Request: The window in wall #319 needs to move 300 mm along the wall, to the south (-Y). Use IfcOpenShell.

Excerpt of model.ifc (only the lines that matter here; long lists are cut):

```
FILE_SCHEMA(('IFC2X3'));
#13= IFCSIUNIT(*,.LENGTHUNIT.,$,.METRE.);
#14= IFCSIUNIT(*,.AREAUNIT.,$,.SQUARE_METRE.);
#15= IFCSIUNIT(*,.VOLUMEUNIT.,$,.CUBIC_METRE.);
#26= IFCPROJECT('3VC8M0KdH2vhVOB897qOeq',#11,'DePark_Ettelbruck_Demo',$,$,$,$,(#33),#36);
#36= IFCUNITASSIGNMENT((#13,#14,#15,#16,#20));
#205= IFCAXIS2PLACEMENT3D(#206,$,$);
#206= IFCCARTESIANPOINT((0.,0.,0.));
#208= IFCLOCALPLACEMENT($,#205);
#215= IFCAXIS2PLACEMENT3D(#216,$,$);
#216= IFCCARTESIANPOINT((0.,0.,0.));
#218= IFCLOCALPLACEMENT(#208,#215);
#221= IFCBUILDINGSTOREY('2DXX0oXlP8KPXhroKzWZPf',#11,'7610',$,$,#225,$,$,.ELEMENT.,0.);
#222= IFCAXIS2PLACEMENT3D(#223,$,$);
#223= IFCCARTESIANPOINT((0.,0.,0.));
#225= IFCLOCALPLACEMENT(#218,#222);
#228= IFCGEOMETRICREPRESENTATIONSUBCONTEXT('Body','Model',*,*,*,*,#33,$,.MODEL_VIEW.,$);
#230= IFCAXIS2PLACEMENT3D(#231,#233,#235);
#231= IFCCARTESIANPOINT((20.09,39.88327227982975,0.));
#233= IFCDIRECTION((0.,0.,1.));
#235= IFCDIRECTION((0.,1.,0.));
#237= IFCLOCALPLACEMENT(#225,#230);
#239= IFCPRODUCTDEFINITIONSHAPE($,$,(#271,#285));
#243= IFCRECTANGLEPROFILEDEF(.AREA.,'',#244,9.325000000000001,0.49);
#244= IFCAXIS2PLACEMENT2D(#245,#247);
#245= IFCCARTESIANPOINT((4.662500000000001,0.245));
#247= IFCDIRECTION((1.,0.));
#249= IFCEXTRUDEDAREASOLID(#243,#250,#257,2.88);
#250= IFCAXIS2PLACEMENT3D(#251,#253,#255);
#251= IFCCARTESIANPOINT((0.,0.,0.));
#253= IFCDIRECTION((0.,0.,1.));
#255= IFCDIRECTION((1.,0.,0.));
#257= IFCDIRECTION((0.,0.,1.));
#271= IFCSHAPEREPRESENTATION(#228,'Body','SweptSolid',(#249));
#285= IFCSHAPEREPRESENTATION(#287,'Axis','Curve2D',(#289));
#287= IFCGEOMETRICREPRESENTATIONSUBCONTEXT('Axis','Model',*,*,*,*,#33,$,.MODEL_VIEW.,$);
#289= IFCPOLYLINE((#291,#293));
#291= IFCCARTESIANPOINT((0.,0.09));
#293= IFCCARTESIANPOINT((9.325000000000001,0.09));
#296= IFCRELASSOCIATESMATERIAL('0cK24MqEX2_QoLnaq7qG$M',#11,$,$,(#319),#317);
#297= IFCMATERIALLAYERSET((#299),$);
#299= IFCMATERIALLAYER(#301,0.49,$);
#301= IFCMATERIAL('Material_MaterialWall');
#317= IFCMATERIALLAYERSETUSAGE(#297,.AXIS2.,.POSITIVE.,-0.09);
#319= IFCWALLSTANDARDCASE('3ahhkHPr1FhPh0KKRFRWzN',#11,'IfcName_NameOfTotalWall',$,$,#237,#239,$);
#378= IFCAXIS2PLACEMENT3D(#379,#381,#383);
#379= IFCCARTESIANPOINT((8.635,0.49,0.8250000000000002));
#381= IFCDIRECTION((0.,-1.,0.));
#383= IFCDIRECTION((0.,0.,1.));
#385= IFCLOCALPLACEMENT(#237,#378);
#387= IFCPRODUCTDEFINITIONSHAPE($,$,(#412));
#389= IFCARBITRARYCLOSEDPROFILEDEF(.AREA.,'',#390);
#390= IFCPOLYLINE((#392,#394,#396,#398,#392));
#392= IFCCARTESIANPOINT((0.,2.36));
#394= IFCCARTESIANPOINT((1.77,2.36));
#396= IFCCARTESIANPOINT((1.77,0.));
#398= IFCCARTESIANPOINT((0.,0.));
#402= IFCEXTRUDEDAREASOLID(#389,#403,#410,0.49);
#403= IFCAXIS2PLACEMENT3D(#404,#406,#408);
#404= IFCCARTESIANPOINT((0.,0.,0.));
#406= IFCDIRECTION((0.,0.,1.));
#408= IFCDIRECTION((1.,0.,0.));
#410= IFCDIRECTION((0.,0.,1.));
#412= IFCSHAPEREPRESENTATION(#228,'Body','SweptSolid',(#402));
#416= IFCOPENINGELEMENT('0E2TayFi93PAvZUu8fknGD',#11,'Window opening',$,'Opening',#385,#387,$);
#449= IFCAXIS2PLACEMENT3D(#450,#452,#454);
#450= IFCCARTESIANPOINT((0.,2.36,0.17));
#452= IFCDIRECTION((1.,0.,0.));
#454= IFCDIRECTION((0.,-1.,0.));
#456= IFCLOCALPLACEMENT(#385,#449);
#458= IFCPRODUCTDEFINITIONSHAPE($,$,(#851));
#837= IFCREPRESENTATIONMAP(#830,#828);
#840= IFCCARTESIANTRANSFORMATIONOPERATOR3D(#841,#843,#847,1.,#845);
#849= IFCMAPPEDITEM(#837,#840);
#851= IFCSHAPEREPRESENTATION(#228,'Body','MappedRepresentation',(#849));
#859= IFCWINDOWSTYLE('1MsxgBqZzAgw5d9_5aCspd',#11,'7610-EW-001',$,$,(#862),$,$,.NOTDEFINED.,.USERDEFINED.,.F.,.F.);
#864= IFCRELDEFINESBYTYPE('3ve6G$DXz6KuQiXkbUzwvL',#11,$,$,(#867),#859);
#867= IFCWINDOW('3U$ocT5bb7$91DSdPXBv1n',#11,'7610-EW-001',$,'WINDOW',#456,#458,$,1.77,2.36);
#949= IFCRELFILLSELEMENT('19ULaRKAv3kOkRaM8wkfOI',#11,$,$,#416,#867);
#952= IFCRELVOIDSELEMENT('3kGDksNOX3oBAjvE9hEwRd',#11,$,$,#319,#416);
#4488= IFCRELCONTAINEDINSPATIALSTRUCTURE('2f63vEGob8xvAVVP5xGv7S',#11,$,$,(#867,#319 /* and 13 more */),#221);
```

```python
import ifcopenshell
import ifcopenshell.api.geometry
import ifcopenshell.util.placement

model = ifcopenshell.open("model.ifc")

window = model.by_guid("3U$ocT5bb7$91DSdPXBv1n")
opening = window.FillsVoids[0].RelatingOpeningElement
wall = opening.VoidsElements[0].RelatingBuildingElement

wall_matrix = ifcopenshell.util.placement.get_local_placement(wall.ObjectPlacement)
shift = wall_matrix[:3, 0] * -0.3
before = ifcopenshell.util.placement.get_local_placement(window.ObjectPlacement)[:3, 3].copy()

# The window is placed relative to its opening, so it follows when the opening moves.
matrix = ifcopenshell.util.placement.get_local_placement(opening.ObjectPlacement)
matrix[:3, 3] += shift
ifcopenshell.api.geometry.edit_object_placement(
    model, product=opening, matrix=matrix, is_si=False, should_transform_children=True
)

after = ifcopenshell.util.placement.get_local_placement(window.ObjectPlacement)[:3, 3]
print("window moved by", (after - before).round(3) + 0.0)

model.write("model_v2.ifc")
```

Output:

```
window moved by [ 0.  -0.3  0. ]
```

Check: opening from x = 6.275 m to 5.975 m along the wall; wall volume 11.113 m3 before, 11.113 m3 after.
